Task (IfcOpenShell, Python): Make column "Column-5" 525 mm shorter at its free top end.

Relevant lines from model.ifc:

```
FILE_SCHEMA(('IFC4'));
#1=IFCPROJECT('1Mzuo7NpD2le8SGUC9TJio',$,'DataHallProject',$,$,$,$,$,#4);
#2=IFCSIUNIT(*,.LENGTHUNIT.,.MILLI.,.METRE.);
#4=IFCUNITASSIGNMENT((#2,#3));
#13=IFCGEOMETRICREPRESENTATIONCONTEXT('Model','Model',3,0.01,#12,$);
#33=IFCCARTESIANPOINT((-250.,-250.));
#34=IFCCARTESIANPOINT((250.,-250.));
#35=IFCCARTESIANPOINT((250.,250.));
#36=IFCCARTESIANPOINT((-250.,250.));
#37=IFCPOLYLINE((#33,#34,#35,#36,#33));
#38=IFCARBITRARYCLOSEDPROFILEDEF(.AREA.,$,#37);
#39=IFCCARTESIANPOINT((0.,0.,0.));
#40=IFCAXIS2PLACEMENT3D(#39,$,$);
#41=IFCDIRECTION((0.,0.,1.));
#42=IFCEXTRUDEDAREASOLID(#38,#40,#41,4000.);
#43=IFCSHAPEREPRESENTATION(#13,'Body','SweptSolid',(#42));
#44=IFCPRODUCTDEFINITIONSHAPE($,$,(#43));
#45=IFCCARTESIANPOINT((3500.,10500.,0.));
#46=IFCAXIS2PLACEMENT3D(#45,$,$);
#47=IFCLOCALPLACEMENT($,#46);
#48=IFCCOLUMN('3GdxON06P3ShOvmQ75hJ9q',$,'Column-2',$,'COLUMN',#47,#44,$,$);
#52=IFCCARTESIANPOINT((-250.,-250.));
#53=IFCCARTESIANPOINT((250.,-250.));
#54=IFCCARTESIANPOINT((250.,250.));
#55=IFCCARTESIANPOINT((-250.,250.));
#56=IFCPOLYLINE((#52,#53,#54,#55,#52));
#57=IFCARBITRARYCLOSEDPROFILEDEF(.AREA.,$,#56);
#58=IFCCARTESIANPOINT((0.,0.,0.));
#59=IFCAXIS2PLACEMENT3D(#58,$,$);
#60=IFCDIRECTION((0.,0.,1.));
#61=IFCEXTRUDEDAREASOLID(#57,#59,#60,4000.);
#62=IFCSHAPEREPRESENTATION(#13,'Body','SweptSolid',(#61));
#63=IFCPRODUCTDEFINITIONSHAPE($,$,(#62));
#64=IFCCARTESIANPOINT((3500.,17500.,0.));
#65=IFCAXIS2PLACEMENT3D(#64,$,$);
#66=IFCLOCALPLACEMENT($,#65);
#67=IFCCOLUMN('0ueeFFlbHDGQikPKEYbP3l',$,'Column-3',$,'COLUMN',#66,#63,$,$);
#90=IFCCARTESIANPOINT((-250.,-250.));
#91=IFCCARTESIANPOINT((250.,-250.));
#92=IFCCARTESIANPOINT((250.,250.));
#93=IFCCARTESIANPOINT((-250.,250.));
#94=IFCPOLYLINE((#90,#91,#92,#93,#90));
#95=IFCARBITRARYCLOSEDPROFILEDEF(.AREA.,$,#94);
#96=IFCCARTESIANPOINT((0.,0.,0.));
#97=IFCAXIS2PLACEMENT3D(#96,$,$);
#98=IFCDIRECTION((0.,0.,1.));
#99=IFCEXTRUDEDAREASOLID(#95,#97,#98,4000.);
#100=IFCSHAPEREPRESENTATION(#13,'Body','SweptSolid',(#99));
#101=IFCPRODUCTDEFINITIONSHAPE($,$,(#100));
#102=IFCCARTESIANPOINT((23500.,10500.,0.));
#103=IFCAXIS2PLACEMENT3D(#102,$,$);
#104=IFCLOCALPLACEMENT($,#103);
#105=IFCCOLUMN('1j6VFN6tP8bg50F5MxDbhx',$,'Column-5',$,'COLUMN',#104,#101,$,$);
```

```python
import ifcopenshell

model = ifcopenshell.open("model.ifc")

member = model.by_guid("1j6VFN6tP8bg50F5MxDbhx")
change = -525.0

# The extrusion runs towards the end named, so only its depth changes.
body = next(r for r in member.Representation.Representations if r.RepresentationIdentifier == "Body")
solid = body.Items[0]
old_length = solid.Depth
solid.Depth += change

print(f"length {old_length:g} -> {solid.Depth:g}")

model.write("model-out.ifc")
```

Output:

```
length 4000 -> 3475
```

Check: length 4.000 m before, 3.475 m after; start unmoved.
